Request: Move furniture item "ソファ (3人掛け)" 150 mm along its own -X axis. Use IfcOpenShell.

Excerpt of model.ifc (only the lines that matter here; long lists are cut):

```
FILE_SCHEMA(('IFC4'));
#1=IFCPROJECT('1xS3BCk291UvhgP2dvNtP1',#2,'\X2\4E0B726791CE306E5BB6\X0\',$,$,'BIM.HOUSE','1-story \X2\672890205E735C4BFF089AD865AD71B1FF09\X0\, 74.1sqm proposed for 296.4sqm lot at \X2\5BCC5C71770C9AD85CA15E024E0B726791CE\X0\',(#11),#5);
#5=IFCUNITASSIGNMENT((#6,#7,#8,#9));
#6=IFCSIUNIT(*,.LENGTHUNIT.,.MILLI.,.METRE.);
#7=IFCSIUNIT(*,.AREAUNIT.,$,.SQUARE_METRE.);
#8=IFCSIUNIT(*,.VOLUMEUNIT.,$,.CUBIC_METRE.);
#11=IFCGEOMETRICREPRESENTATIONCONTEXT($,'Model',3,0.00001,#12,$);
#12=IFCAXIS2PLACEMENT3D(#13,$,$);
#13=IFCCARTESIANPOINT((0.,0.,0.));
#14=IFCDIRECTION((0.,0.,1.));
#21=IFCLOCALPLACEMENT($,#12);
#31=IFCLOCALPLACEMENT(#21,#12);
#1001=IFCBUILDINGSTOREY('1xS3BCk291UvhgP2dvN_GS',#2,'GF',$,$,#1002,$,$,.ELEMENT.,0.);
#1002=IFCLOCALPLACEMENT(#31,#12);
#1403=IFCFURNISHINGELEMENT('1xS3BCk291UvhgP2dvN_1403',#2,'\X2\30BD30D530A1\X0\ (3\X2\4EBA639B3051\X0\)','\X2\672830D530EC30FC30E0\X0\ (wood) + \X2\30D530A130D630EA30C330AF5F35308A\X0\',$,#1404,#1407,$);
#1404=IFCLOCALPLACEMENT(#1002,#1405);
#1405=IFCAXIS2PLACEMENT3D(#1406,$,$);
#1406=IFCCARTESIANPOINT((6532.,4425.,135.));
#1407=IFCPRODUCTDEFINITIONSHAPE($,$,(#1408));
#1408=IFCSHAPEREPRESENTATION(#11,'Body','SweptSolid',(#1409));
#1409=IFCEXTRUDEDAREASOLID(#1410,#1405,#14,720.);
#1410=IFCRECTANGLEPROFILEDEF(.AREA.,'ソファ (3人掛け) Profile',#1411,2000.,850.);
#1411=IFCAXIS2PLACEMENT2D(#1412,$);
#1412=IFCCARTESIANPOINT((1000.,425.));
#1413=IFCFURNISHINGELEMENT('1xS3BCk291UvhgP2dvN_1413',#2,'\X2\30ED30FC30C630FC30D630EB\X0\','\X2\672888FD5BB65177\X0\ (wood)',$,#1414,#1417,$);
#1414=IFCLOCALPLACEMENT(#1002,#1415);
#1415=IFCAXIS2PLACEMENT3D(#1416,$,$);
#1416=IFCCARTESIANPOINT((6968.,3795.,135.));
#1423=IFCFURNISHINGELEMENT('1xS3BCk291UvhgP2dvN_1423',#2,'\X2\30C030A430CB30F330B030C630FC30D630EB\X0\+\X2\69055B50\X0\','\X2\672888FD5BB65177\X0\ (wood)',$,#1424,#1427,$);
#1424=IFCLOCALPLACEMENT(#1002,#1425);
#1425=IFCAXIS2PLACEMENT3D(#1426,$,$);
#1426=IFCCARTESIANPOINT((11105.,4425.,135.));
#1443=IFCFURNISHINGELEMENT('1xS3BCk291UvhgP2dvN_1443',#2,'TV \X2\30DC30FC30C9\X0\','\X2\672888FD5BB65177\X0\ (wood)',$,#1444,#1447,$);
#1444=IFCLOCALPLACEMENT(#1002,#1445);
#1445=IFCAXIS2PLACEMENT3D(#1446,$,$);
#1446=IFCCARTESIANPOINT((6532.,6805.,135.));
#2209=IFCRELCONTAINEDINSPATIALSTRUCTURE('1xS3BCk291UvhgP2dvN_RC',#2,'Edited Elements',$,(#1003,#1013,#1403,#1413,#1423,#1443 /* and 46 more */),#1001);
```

```python
import ifcopenshell
import ifcopenshell.api.geometry
import ifcopenshell.util.placement

model = ifcopenshell.open("model.ifc")

item = model.by_guid("1xS3BCk291UvhgP2dvN_1403")
matrix = ifcopenshell.util.placement.get_local_placement(item.ObjectPlacement)
matrix[:3, 3] -= matrix[:3, 0] * 150.0
ifcopenshell.api.geometry.edit_object_placement(model, product=item, matrix=matrix, is_si=False)

print(ifcopenshell.util.placement.get_local_placement(item.ObjectPlacement).round(3) + 0.0)

model.write("model-out.ifc")
```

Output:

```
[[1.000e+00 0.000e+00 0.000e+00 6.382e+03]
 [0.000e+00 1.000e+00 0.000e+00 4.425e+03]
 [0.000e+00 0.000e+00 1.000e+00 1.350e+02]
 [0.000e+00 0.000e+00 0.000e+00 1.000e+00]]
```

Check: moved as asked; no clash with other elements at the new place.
